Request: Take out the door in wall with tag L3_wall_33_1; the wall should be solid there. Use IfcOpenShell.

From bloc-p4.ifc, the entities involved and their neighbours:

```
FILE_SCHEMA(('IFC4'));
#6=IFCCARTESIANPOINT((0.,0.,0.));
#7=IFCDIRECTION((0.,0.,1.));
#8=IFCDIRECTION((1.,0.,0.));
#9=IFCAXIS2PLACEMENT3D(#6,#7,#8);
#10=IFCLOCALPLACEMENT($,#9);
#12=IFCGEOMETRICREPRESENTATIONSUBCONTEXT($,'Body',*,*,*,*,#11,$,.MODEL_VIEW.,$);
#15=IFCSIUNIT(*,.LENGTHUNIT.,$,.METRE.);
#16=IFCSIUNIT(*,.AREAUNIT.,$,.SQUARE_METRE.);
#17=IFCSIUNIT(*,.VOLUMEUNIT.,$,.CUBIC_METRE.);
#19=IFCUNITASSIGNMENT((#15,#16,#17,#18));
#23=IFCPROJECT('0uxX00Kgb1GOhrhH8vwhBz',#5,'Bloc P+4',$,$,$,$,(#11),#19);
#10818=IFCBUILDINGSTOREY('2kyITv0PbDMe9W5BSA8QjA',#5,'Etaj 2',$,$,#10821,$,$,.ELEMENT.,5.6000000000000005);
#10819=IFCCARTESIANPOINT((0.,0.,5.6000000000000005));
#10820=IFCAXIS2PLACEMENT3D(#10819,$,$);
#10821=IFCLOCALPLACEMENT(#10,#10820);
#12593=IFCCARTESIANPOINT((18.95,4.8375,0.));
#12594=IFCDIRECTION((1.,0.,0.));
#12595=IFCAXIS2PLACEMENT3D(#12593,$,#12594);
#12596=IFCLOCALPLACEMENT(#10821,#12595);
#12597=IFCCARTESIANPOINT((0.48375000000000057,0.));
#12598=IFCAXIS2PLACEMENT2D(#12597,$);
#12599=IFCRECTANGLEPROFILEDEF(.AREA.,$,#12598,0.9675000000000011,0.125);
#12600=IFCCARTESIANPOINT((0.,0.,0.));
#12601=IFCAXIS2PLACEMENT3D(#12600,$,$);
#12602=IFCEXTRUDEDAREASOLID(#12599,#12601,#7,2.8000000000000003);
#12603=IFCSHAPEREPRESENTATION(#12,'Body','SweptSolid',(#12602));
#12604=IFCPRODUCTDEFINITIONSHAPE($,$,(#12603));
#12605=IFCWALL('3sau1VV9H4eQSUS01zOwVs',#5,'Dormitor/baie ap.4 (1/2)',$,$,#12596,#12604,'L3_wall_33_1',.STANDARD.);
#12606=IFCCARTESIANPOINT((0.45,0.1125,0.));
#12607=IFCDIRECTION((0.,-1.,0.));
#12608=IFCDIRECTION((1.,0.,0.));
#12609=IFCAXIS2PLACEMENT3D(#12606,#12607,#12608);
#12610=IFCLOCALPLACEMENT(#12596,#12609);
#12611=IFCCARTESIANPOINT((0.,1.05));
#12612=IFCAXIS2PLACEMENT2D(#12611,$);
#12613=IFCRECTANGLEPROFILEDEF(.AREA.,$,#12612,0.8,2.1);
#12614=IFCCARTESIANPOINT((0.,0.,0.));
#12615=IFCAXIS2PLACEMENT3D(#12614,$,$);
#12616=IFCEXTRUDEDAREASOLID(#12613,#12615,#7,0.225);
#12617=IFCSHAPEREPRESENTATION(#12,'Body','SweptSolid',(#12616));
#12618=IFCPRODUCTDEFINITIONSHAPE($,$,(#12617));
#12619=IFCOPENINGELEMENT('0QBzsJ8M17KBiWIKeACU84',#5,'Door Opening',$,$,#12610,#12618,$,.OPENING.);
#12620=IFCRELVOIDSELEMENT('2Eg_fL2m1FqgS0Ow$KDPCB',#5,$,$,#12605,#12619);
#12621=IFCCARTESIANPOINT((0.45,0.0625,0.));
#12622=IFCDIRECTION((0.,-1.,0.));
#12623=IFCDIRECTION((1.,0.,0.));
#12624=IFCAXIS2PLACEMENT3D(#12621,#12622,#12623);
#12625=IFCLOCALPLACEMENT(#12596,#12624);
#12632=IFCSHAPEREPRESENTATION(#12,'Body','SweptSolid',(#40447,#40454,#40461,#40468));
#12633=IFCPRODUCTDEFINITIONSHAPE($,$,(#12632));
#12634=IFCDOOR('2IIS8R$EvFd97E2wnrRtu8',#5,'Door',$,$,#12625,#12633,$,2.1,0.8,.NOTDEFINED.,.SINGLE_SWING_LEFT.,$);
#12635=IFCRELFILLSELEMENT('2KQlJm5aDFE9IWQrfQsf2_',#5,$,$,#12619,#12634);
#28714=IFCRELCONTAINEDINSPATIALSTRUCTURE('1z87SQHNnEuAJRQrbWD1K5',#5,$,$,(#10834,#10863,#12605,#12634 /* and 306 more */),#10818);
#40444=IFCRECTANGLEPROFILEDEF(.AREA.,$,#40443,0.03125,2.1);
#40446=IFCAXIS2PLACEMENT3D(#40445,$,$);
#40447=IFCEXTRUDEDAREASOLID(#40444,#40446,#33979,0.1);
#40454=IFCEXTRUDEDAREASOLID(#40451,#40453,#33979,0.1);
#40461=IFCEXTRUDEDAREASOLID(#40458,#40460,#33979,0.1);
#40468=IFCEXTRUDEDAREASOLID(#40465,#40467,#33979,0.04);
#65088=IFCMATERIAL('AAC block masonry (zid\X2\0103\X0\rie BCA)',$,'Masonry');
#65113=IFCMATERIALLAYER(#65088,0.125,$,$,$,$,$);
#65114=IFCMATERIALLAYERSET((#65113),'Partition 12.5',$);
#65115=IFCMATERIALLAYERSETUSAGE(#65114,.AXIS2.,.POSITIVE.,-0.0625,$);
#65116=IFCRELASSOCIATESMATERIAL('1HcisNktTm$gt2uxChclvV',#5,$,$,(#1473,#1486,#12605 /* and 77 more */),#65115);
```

```python
import ifcopenshell
import ifcopenshell.api.feature
import ifcopenshell.api.root
import ifcopenshell.geom
import ifcopenshell.util.shape

model = ifcopenshell.open("bloc-p4.ifc")
settings = ifcopenshell.geom.settings()


def volume(element):
    """Net volume in cubic metres, openings subtracted."""
    shape = ifcopenshell.geom.create_shape(settings, element)
    return ifcopenshell.util.shape.get_volume(shape.geometry)


door = model.by_guid("2IIS8R$EvFd97E2wnrRtu8")
opening = door.FillsVoids[0].RelatingOpeningElement
wall = opening.VoidsElements[0].RelatingBuildingElement
before = volume(wall)

ifcopenshell.api.root.remove_product(model, product=door)
ifcopenshell.api.feature.remove_feature(model, feature=opening)

after = volume(wall)

print(f"wall volume {before:.3f} -> {after:.3f} m3")

model.write("bloc-p4-out.ifc")
```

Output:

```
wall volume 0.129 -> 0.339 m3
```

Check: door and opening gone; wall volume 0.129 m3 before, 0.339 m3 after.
